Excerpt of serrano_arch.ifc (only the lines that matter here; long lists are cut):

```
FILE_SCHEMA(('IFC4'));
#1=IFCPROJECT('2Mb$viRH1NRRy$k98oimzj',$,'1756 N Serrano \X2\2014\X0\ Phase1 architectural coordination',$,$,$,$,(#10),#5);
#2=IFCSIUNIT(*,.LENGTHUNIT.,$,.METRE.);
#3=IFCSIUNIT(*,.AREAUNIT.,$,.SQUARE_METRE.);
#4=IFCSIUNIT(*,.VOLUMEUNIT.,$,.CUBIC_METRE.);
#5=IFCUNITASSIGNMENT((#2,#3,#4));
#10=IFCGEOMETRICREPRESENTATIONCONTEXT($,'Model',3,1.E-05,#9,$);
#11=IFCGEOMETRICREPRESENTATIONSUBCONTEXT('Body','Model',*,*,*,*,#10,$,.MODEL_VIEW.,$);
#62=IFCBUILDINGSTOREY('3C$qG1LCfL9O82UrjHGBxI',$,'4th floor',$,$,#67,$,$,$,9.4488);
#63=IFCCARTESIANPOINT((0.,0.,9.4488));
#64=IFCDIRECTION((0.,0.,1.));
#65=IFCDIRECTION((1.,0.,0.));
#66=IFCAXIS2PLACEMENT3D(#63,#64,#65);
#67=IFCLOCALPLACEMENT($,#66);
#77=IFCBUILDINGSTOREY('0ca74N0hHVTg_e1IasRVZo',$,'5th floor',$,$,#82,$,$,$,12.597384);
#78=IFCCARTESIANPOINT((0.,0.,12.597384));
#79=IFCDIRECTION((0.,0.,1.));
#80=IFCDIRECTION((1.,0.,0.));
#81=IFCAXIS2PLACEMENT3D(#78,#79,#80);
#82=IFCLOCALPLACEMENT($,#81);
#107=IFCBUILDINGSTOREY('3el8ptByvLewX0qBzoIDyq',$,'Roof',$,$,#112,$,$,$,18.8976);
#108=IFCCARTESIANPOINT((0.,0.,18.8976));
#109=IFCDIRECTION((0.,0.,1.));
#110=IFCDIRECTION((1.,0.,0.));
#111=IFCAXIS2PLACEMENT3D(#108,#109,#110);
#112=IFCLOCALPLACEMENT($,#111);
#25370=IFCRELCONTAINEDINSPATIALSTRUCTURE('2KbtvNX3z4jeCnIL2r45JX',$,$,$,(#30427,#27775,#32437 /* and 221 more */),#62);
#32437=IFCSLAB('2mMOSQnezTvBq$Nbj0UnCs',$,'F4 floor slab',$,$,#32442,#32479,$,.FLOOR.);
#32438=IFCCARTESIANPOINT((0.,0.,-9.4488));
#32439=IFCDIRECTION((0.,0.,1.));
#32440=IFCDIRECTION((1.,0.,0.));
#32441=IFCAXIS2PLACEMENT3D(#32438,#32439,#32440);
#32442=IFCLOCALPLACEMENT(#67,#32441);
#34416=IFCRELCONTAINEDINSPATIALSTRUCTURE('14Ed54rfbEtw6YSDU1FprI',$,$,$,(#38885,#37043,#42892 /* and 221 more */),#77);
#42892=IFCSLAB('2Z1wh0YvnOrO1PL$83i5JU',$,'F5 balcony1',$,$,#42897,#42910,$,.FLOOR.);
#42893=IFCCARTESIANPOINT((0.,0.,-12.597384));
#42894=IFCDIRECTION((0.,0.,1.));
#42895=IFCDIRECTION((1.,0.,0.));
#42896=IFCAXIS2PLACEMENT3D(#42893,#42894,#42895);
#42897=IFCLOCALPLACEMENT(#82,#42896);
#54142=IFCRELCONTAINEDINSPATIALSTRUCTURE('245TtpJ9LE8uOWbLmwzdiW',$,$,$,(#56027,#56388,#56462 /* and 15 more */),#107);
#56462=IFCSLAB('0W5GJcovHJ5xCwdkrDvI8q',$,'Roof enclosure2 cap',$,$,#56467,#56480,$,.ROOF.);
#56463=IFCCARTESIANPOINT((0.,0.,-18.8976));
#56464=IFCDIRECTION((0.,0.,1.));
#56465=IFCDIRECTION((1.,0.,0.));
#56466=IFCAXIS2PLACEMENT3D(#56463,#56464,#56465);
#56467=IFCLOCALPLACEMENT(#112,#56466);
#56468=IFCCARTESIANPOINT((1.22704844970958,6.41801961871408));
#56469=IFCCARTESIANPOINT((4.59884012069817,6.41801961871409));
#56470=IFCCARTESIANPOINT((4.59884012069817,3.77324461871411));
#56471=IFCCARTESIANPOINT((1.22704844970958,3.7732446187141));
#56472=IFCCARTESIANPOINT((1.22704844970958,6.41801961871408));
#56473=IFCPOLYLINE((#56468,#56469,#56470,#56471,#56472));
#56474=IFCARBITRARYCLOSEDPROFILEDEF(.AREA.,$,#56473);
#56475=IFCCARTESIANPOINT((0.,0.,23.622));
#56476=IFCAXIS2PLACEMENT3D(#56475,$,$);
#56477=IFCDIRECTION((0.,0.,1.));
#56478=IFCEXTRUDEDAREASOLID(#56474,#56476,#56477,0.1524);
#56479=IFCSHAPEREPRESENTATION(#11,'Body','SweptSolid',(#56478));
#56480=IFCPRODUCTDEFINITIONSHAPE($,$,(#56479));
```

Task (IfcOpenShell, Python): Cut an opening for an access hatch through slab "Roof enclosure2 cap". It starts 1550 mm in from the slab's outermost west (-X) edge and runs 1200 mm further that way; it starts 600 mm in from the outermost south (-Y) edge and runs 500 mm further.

```python
import numpy as np
import ifcopenshell
import ifcopenshell.api.feature
import ifcopenshell.api.geometry
import ifcopenshell.api.root
import ifcopenshell.geom
import ifcopenshell.util.placement
import ifcopenshell.util.representation
import ifcopenshell.util.shape
import ifcopenshell.util.unit

model = ifcopenshell.open("serrano_arch.ifc")
unit_scale = ifcopenshell.util.unit.calculate_unit_scale(model)
settings = ifcopenshell.geom.settings()


def volume(element):
    """Net volume in cubic metres, openings subtracted."""
    shape = ifcopenshell.geom.create_shape(settings, element)
    return ifcopenshell.util.shape.get_volume(shape.geometry)


slab = model.by_id(56462)
before = volume(slab)

# Extent in the slab's own axes, in metres. The edges named are its -X and -Y sides.
slab_shape = ifcopenshell.geom.create_shape(settings, slab)
vertices = ifcopenshell.util.shape.get_vertices(slab_shape.geometry)
x_min, y_min, bottom = vertices.min(axis=0)
top = vertices[:, 2].max()

opening = ifcopenshell.api.root.create_entity(model, ifc_class="IfcOpeningElement", name="Access hatch opening", predefined_type="OPENING")
context = ifcopenshell.util.representation.get_context(model, "Model", "Body", "MODEL_VIEW")
width, depth = 1.2, 0.5
outline = [(0.0, 0.0), (width, 0.0), (width, depth), (0.0, depth), (0.0, 0.0)]
# Overshoot both faces by 50 mm so the cut is clean.
shape = ifcopenshell.api.geometry.add_slab_representation(
    model, context=context, depth=top - bottom + 0.1, polyline=outline
)
ifcopenshell.api.geometry.assign_representation(model, product=opening, representation=shape)

matrix = ifcopenshell.util.placement.get_local_placement(slab.ObjectPlacement)
matrix[:, 3] = matrix @ np.append(np.array([x_min + 1.55, y_min + 0.6, bottom - 0.05]) / unit_scale, 1.0)
ifcopenshell.api.geometry.edit_object_placement(model, product=opening, matrix=matrix, is_si=False)
ifcopenshell.api.feature.add_feature(model, feature=opening, element=slab)

after = volume(slab)

print(f"slab volume {before:.3f} -> {after:.3f} m3")

model.write("serrano_arch-out.ifc")
```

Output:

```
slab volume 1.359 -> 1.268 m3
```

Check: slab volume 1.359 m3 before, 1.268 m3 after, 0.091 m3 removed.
